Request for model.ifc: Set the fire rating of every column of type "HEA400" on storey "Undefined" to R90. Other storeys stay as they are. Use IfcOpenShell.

First a look at what the model holds.

```python
import ifcopenshell
import ifcopenshell.util.element

model = ifcopenshell.open("model.ifc")
print(model.schema)
storey = next(s for s in model.by_type("IfcBuildingStorey") if s.Name == "Undefined")
columns = [e for e in ifcopenshell.util.element.get_decomposition(storey) if e.is_a("IfcColumn")]
seen = {}
for e in columns:
    element_type = ifcopenshell.util.element.get_type(e)
    key = (element_type.Name if element_type != e and element_type else None, ifcopenshell.util.element.get_pset(e, "Pset_ColumnCommon", "FireRating"))
    seen[key] = seen.get(key, 0) + 1
for (name, value), count in sorted(seen.items(), key=str):
    print(count, "x", name, "|", value)
```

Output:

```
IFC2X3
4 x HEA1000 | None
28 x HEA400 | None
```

```python
import ifcopenshell
import ifcopenshell.api.pset
import ifcopenshell.util.element

model = ifcopenshell.open("model.ifc")

storey = next(s for s in model.by_type("IfcBuildingStorey") if s.Name == "Undefined")
columns = [e for e in ifcopenshell.util.element.get_decomposition(storey) if e.is_a("IfcColumn")]

count = 0
for e in columns:
    element_type = ifcopenshell.util.element.get_type(e)
    if element_type in (None, e) or element_type.Name != "HEA400":
        continue
    found = ifcopenshell.util.element.get_pset(e, "Pset_ColumnCommon", should_inherit=False)
    if found:
        pset = model.by_id(found["id"])
        if len(ifcopenshell.util.element.get_elements_by_pset(pset)) > 1:
            pset = ifcopenshell.api.pset.unshare_pset(model, products=[e], pset=pset)[0]
    else:
        pset = ifcopenshell.api.pset.add_pset(model, product=e, name="Pset_ColumnCommon")
    ifcopenshell.api.pset.edit_pset(model, pset=pset, properties={"FireRating": "R90"})
    count += 1

print(count, "columns updated")

model.write("model_v2.ifc")
```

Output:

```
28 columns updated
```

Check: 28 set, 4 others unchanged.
